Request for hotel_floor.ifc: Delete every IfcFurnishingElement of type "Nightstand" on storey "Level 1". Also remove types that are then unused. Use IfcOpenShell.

First a look at what the model holds.

```python
import ifcopenshell
import ifcopenshell.util.element

model = ifcopenshell.open("hotel_floor.ifc")
print(model.schema)
storey = next(s for s in model.by_type("IfcBuildingStorey") if s.Name == "Level 1")
furniture = [e for e in ifcopenshell.util.element.get_decomposition(storey) if e.is_a("IfcFurnishingElement")]
seen = {}
for e in furniture:
    element_type = ifcopenshell.util.element.get_type(e)
    name = element_type.Name if element_type not in (None, e) else None
    seen[name] = seen.get(name, 0) + 1
for name, count in sorted(seen.items(), key=str):
    print(count, "x", name)
```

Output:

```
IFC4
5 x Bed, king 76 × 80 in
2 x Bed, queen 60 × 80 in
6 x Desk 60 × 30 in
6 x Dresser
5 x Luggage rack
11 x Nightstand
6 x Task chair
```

```python
import ifcopenshell
import ifcopenshell.api.root
import ifcopenshell.util.element

model = ifcopenshell.open("hotel_floor.ifc")

storey = next(s for s in model.by_type("IfcBuildingStorey") if s.Name == "Level 1")
furniture = [e for e in ifcopenshell.util.element.get_decomposition(storey) if e.is_a("IfcFurnishingElement")]
targets = [e for e in furniture if (t := ifcopenshell.util.element.get_type(e)) not in (None, e) and t.Name == "Nightstand"]
types = {ifcopenshell.util.element.get_type(e) for e in targets} - {None, *targets}

for e in targets:
    ifcopenshell.api.root.remove_product(model, product=e)
print(len(targets), "removed")

unused = [t for t in types if not ifcopenshell.util.element.get_types(t)]
for t in unused:
    ifcopenshell.api.root.remove_product(model, product=t)
print(len(unused), "unused types removed")

model.write("hotel_floor_rev.ifc")
```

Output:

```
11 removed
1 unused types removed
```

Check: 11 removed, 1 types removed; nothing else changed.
